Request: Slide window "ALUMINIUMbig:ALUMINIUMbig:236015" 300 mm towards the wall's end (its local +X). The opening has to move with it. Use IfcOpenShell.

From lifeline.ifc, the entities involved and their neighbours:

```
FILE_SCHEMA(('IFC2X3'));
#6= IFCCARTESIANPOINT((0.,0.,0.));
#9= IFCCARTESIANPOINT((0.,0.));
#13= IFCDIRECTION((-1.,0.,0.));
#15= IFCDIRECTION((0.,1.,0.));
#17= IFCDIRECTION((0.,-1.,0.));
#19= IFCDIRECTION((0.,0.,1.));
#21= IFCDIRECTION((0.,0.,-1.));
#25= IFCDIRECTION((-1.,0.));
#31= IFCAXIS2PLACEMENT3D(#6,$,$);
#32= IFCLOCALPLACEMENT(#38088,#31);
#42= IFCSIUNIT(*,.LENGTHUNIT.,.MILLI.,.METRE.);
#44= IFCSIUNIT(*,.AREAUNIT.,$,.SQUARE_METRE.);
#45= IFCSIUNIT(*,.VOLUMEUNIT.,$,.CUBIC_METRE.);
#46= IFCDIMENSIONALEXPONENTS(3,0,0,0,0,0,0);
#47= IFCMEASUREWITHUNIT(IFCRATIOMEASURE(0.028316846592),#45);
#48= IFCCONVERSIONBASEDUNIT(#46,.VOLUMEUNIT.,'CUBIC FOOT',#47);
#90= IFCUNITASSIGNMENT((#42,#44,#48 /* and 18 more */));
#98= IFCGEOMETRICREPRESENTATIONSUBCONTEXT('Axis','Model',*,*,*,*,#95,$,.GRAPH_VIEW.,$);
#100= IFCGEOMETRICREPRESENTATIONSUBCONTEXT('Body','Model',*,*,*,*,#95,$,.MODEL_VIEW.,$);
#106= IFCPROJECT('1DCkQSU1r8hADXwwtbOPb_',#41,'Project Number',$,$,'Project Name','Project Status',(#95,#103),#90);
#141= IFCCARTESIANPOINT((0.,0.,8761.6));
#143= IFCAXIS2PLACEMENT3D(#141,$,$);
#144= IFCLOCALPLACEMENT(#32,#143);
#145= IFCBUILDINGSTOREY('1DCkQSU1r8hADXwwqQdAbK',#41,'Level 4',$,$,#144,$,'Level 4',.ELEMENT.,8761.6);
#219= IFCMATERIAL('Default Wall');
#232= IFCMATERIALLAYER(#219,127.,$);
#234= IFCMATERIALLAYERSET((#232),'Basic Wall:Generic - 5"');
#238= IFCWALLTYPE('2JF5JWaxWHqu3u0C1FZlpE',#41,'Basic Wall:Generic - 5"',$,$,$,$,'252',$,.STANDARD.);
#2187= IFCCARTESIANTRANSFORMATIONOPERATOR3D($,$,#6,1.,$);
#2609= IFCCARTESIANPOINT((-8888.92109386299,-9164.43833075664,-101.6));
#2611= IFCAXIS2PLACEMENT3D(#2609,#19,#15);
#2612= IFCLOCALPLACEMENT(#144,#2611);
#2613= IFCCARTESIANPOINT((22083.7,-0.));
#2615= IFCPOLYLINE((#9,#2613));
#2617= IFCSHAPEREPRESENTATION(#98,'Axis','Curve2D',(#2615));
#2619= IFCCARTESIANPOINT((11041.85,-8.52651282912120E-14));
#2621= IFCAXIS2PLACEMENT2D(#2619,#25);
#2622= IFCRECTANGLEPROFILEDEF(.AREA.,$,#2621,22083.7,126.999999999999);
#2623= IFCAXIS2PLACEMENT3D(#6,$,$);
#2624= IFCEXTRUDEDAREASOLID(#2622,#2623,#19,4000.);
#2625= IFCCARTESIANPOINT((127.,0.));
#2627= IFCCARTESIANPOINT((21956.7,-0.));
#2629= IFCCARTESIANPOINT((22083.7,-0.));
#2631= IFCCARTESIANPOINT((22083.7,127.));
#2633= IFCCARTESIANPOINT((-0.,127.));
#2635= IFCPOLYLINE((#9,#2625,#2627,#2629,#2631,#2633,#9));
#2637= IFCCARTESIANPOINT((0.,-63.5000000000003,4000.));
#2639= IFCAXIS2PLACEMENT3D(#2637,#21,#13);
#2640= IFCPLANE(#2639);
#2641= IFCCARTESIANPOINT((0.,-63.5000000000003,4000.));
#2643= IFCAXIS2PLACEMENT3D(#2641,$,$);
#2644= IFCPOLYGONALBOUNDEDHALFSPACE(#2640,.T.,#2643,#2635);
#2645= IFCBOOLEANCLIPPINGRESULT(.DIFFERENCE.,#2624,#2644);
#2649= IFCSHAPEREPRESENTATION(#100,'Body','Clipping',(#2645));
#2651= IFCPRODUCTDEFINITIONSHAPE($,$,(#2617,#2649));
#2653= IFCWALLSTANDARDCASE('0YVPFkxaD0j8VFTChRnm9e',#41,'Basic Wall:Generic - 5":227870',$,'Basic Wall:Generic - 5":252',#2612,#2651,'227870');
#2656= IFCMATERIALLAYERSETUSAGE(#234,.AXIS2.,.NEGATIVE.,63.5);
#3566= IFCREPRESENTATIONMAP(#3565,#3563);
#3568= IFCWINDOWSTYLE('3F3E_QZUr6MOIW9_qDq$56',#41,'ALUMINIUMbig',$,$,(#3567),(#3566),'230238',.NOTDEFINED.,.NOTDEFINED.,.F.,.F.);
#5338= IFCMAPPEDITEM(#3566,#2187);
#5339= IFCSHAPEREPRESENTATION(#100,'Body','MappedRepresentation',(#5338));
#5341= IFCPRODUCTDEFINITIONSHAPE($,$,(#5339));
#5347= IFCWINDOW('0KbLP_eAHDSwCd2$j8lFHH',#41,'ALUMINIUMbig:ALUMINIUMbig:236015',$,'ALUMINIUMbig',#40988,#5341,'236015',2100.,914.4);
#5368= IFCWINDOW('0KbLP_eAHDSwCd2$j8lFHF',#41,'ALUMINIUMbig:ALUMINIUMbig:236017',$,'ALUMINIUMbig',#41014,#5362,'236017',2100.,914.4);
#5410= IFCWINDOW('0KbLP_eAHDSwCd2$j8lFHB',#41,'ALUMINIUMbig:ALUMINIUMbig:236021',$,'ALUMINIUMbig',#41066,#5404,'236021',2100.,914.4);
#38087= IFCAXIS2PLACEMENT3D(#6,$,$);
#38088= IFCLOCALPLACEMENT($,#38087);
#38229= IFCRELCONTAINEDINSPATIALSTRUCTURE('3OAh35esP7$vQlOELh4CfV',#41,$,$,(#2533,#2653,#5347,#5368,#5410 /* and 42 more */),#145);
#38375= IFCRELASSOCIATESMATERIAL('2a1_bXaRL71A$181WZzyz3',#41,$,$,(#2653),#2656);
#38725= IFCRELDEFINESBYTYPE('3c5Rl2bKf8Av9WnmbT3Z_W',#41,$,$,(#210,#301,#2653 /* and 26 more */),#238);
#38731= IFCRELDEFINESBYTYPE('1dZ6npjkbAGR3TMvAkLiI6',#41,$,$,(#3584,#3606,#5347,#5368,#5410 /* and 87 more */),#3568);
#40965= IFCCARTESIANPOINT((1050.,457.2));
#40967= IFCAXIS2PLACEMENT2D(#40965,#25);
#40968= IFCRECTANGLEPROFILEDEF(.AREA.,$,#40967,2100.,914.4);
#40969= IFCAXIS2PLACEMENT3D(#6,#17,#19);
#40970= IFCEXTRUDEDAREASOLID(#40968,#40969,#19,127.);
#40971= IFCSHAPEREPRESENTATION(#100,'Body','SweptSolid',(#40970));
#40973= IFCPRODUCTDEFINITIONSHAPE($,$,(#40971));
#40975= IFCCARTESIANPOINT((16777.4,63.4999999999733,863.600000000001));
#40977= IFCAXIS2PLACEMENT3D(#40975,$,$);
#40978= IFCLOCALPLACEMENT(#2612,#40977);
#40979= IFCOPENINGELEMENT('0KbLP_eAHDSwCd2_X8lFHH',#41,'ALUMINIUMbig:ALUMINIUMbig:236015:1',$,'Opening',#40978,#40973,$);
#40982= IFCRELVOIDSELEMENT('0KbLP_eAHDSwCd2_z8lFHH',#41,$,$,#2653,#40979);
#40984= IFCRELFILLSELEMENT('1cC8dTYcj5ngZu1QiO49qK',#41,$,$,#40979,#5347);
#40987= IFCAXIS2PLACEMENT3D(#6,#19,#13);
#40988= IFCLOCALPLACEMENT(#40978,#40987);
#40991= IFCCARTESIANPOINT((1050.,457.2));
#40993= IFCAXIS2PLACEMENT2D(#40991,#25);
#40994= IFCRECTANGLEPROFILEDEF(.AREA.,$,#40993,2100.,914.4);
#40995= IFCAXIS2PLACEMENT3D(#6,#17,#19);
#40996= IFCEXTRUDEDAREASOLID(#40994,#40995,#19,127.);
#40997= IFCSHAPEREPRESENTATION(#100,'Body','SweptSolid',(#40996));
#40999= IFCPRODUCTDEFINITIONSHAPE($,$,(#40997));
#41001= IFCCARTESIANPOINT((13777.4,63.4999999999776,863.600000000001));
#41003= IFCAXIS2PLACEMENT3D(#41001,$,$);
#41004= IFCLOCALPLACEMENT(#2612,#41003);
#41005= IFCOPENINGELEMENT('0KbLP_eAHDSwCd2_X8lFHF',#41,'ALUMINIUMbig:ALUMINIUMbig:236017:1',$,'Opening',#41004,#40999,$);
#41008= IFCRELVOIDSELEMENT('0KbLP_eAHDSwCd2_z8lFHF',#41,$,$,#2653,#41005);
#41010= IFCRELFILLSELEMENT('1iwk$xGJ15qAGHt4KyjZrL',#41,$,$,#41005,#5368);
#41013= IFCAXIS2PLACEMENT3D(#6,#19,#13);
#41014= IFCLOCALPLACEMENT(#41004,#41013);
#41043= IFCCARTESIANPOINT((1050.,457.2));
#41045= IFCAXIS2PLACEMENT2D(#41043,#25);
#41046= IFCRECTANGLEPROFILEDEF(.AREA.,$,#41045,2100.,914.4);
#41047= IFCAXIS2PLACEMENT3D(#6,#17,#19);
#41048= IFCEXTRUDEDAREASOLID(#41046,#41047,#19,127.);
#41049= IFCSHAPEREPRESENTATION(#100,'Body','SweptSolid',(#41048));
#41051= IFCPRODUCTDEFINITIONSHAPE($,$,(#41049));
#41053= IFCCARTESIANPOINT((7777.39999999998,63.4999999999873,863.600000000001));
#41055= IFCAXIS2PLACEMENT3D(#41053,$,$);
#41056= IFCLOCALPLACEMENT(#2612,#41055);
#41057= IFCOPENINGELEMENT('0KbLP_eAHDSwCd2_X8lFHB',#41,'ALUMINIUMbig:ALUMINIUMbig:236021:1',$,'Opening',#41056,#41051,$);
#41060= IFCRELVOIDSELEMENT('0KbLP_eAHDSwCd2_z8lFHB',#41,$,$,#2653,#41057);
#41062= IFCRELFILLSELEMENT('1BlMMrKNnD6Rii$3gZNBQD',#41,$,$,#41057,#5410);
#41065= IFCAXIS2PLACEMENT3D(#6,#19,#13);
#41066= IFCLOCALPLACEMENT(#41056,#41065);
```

```python
import ifcopenshell
import ifcopenshell.api.geometry
import ifcopenshell.util.placement
import ifcopenshell.util.unit

model = ifcopenshell.open("lifeline.ifc")
unit_scale = ifcopenshell.util.unit.calculate_unit_scale(model)

window = model.by_guid("0KbLP_eAHDSwCd2$j8lFHH")
opening = window.FillsVoids[0].RelatingOpeningElement
wall = opening.VoidsElements[0].RelatingBuildingElement

wall_matrix = ifcopenshell.util.placement.get_local_placement(wall.ObjectPlacement)
shift = wall_matrix[:3, 0] * 0.3 / unit_scale
before = ifcopenshell.util.placement.get_local_placement(window.ObjectPlacement)[:3, 3].copy()

# The window is placed relative to its opening, so it follows when the opening moves.
matrix = ifcopenshell.util.placement.get_local_placement(opening.ObjectPlacement)
matrix[:3, 3] += shift
ifcopenshell.api.geometry.edit_object_placement(
    model, product=opening, matrix=matrix, is_si=False, should_transform_children=True
)

after = ifcopenshell.util.placement.get_local_placement(window.ObjectPlacement)[:3, 3]
print("window moved by", (after - before).round(3) + 0.0)

model.write("lifeline-out.ifc")
```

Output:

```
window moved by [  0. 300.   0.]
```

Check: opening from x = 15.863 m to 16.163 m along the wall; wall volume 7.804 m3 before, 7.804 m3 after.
